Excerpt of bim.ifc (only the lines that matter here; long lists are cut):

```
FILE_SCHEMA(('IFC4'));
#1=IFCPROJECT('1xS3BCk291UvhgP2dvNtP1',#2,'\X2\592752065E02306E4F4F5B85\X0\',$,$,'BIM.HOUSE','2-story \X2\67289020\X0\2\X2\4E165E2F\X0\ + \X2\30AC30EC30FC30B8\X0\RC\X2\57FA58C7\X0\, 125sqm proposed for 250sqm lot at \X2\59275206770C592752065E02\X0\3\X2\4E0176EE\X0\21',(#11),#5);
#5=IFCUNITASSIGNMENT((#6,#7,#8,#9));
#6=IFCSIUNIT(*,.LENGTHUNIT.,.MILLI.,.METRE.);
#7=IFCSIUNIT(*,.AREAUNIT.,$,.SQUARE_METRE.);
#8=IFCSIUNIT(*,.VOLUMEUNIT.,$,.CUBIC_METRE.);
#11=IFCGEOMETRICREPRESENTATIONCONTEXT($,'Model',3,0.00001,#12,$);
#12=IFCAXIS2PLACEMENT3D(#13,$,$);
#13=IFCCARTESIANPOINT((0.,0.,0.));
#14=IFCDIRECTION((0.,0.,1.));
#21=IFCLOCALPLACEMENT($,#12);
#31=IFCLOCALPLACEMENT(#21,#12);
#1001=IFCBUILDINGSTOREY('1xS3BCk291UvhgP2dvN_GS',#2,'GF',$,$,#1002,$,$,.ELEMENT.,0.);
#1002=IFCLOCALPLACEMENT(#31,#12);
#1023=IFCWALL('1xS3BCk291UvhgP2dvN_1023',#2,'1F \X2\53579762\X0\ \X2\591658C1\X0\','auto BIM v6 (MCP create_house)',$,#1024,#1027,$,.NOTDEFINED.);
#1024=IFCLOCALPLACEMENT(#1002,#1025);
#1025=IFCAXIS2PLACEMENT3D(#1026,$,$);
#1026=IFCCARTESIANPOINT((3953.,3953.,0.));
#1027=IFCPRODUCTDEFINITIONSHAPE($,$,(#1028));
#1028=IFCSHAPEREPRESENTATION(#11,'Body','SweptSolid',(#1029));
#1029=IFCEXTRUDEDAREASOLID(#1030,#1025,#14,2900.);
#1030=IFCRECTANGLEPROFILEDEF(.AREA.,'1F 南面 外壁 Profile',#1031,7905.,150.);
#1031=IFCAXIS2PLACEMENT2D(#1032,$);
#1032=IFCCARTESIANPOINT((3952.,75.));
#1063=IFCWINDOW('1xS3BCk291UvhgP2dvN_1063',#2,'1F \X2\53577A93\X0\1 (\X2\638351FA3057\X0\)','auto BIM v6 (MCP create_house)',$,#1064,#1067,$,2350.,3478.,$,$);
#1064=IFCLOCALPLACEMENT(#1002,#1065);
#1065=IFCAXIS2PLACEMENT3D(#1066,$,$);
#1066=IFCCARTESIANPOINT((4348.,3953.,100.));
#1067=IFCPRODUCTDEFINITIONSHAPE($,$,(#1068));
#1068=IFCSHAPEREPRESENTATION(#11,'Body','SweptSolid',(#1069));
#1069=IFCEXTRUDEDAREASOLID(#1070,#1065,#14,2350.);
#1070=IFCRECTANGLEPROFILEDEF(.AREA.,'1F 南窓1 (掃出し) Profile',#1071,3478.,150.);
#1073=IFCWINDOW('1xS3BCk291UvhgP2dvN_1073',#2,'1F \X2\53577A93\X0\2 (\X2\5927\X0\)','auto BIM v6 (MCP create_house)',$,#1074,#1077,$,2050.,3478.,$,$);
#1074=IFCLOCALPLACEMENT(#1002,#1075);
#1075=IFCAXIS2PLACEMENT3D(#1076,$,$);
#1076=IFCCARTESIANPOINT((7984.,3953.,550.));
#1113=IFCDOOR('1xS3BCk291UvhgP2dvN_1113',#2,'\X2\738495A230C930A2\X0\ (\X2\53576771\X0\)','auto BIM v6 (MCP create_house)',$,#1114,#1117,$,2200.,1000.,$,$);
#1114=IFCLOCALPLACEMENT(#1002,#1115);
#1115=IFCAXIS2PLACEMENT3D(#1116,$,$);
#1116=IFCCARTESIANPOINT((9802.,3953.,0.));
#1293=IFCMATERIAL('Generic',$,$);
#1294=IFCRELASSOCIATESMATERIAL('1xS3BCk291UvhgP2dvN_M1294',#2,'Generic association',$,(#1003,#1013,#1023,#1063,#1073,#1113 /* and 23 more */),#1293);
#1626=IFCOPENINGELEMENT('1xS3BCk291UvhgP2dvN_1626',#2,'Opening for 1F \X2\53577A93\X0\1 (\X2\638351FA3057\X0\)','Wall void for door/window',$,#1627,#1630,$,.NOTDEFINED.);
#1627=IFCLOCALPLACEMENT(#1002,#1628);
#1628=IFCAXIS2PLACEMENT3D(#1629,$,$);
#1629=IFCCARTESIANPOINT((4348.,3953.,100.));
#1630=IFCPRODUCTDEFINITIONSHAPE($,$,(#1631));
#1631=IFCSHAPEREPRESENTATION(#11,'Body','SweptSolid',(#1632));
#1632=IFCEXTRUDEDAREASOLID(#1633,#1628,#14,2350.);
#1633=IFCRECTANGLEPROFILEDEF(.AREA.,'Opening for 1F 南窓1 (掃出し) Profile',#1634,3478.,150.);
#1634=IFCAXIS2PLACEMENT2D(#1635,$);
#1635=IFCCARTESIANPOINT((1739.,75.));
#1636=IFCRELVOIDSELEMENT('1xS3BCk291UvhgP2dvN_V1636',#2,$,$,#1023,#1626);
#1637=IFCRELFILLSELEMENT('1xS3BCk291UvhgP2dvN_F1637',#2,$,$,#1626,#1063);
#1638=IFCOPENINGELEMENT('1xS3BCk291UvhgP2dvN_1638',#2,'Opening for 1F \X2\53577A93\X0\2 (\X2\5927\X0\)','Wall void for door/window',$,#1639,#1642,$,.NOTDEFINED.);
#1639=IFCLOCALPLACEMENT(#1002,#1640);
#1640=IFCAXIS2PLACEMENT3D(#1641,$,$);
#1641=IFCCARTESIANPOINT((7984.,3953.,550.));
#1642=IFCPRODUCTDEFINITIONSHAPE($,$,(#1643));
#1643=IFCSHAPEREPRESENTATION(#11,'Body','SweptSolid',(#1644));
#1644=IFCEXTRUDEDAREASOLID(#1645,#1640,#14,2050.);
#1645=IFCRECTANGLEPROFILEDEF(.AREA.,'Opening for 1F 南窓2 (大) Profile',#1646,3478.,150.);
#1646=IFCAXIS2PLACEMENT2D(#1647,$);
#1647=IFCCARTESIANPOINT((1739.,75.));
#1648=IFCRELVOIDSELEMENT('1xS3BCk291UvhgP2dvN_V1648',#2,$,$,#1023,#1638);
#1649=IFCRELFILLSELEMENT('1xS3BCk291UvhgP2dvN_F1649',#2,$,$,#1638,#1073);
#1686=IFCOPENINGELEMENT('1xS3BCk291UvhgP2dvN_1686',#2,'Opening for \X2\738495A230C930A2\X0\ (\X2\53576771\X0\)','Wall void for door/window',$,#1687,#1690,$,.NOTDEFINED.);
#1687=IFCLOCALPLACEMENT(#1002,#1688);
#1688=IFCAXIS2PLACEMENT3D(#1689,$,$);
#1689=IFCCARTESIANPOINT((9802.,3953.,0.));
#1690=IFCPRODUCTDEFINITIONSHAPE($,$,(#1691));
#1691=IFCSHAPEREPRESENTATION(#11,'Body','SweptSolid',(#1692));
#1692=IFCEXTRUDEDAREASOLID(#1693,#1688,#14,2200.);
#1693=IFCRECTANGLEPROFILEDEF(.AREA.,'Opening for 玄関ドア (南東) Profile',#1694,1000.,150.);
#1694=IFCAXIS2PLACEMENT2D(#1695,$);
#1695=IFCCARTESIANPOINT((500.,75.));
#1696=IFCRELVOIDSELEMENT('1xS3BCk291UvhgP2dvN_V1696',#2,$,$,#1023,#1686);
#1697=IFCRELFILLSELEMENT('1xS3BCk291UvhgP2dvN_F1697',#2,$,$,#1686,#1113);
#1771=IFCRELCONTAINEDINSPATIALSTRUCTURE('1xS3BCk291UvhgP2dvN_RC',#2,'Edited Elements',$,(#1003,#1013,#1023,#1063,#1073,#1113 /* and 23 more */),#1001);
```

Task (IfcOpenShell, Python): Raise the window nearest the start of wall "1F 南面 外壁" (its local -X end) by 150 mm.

```python
import numpy as np
import ifcopenshell
import ifcopenshell.api.geometry
import ifcopenshell.util.placement
import ifcopenshell.util.unit

model = ifcopenshell.open("bim.ifc")
unit_scale = ifcopenshell.util.unit.calculate_unit_scale(model)

window = model.by_guid("1xS3BCk291UvhgP2dvN_1063")
opening = window.FillsVoids[0].RelatingOpeningElement
dz = 0.15 / unit_scale

shift = np.array([0.0, 0.0, dz])
# The window is not placed relative to its opening, so move both.
for product in (opening, window):
    matrix = ifcopenshell.util.placement.get_local_placement(product.ObjectPlacement)
    matrix[:3, 3] += shift
    ifcopenshell.api.geometry.edit_object_placement(model, product=product, matrix=matrix, is_si=False)

print(f"moved by {dz * unit_scale:+.3f} m")

model.write("bim_edited.ifc")
```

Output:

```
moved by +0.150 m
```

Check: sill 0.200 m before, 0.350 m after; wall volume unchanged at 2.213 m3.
